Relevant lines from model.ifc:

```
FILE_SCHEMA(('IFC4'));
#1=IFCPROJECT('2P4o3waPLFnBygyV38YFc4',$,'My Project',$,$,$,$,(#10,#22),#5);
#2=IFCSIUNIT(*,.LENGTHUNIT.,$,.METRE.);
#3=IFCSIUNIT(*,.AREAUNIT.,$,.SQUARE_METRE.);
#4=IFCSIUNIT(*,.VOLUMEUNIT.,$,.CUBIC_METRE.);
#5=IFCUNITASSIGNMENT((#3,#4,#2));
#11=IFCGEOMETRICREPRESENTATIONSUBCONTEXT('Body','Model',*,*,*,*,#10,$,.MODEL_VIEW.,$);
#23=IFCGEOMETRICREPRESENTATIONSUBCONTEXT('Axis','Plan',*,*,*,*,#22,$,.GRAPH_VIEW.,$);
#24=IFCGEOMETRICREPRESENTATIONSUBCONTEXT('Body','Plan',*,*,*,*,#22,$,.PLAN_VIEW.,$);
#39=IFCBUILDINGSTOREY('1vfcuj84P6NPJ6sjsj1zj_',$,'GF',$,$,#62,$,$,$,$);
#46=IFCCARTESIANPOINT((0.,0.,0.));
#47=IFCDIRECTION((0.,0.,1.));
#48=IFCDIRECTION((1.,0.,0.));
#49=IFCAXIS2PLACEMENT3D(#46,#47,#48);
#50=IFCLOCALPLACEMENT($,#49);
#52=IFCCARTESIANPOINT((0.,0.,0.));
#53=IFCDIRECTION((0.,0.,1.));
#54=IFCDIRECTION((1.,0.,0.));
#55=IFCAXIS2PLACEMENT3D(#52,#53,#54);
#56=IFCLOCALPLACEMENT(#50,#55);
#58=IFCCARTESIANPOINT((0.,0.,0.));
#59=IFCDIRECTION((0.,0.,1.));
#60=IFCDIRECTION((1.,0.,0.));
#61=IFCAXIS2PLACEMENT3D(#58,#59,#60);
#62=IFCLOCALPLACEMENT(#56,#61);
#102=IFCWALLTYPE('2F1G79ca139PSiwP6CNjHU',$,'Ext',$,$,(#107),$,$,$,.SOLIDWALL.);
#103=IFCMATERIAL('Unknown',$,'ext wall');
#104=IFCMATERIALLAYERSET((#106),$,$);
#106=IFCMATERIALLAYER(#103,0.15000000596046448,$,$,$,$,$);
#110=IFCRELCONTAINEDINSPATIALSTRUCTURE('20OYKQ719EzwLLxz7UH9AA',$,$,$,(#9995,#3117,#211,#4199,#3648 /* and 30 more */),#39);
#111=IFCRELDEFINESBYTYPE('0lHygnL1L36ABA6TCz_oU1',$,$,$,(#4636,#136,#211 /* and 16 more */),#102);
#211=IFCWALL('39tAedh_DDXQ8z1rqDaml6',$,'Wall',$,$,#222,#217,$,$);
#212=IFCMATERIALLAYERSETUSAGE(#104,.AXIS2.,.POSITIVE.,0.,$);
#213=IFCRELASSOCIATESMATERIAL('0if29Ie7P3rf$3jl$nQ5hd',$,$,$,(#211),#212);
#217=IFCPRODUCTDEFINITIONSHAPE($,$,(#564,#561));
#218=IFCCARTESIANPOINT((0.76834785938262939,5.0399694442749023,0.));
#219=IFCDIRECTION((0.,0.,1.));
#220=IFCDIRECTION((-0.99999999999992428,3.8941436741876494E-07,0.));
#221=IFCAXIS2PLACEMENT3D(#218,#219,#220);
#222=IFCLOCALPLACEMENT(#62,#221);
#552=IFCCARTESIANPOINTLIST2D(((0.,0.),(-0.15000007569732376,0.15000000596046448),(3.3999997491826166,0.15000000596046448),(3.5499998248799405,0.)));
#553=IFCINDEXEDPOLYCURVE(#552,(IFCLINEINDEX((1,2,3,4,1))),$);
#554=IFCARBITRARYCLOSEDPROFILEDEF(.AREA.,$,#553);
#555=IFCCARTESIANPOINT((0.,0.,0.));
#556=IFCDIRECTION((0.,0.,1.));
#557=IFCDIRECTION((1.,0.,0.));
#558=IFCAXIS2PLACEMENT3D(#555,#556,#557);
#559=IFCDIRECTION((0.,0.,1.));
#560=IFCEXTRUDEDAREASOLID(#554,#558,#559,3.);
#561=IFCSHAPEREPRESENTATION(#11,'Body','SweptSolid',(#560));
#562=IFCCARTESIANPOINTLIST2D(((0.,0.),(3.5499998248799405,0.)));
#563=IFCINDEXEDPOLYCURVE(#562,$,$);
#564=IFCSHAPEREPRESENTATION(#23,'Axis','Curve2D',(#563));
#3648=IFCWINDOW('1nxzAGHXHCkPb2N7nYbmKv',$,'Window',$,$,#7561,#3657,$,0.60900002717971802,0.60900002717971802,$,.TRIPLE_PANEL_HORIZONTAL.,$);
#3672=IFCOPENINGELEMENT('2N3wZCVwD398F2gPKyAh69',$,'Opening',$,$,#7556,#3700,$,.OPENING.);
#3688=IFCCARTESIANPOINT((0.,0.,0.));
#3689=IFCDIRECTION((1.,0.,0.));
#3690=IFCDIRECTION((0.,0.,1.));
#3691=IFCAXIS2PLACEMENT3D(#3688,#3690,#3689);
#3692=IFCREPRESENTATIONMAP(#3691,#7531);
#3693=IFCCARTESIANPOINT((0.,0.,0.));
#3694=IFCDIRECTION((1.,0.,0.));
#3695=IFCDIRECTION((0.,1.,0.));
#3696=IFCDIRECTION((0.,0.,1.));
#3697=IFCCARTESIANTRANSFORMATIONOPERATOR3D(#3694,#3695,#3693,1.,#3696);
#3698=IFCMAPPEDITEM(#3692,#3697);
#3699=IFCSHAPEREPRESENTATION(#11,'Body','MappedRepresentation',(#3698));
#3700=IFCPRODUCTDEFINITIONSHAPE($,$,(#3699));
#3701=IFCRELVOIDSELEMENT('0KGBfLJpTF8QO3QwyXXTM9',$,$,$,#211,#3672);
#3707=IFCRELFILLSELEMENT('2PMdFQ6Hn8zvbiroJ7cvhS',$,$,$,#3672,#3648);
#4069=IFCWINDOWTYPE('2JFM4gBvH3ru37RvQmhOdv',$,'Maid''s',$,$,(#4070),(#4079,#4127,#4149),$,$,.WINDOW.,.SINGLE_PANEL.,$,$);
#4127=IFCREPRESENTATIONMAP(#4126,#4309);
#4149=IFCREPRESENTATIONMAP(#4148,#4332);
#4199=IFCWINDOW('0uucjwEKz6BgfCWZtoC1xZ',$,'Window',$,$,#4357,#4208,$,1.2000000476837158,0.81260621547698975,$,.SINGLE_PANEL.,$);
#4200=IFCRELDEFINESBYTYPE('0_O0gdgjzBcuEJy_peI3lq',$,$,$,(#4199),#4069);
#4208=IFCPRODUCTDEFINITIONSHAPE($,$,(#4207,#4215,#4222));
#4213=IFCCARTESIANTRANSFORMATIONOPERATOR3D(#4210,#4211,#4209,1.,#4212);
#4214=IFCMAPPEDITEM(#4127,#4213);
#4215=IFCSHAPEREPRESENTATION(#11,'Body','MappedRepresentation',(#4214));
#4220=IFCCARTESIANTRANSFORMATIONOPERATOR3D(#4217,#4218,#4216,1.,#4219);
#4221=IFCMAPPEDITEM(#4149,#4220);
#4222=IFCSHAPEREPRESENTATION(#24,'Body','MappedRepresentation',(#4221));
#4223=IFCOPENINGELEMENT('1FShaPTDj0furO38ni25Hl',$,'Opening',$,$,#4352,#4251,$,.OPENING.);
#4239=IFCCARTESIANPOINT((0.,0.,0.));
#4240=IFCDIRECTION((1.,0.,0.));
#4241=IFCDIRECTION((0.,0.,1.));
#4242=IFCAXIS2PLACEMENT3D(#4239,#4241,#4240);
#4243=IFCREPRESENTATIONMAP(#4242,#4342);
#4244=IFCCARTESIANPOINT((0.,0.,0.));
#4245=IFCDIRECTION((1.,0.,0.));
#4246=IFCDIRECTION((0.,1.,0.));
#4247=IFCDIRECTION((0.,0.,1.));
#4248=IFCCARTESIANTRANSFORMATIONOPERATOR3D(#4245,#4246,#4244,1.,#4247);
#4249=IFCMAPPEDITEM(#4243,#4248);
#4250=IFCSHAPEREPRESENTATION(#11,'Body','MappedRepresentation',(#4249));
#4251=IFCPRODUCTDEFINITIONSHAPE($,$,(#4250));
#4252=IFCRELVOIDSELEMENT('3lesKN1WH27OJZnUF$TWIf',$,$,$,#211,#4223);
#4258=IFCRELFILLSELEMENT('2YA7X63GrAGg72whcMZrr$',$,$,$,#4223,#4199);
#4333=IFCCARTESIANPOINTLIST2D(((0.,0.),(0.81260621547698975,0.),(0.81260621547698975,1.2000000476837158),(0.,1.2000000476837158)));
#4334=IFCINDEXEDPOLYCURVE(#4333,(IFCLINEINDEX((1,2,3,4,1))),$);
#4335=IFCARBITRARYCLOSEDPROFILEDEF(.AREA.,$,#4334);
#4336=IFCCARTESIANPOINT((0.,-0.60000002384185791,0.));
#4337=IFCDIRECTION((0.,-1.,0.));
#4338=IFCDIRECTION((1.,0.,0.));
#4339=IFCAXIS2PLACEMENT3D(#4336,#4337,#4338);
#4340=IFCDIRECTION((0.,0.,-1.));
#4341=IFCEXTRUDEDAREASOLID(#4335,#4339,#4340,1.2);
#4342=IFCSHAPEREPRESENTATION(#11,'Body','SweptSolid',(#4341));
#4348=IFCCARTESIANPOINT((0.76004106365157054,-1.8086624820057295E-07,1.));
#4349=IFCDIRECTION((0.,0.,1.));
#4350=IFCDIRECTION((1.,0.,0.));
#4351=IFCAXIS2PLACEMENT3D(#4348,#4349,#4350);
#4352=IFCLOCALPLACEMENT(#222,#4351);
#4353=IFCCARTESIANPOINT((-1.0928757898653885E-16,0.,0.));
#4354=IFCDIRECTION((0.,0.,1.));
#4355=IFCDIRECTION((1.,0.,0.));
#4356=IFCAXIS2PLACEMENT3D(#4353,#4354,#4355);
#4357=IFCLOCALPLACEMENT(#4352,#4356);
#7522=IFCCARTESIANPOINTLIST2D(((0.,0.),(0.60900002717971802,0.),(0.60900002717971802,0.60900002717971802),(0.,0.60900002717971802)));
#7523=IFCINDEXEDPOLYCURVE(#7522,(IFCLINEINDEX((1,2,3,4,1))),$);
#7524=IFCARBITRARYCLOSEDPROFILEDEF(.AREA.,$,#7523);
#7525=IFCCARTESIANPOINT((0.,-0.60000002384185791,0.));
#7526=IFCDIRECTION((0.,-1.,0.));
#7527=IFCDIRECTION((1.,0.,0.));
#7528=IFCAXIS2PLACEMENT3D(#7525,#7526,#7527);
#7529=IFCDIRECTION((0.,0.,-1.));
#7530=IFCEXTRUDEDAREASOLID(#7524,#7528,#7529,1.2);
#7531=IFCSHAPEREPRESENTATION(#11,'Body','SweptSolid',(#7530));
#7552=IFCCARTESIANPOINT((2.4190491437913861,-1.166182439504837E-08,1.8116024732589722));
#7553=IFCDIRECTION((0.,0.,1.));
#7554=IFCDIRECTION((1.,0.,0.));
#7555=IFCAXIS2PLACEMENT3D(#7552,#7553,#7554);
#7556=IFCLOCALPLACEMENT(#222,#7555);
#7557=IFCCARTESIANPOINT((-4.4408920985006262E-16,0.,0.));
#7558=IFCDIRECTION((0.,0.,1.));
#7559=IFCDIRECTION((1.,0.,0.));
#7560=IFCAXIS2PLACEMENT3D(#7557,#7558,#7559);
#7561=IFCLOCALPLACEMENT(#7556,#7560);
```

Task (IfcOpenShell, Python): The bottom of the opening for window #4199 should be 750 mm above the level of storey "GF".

```python
import numpy as np
import ifcopenshell
import ifcopenshell.api.geometry
import ifcopenshell.geom
import ifcopenshell.util.element
import ifcopenshell.util.placement
import ifcopenshell.util.shape
import ifcopenshell.util.unit

model = ifcopenshell.open("model.ifc")
unit_scale = ifcopenshell.util.unit.calculate_unit_scale(model)

window = model.by_id(4199)
opening = window.FillsVoids[0].RelatingOpeningElement
storey = ifcopenshell.util.element.get_container(window, ifc_class="IfcBuildingStorey")
level = ifcopenshell.util.placement.get_local_placement(storey.ObjectPlacement)[2, 3]

# The opening's origin need not be at the sill, so measure its lowest point.
shape = ifcopenshell.geom.create_shape(ifcopenshell.geom.settings(), opening)
bottom = ifcopenshell.util.shape.get_shape_bottom_elevation(shape, shape.geometry) / unit_scale
dz = level + 0.75 - bottom

shift = np.array([0.0, 0.0, dz])
# The window is placed relative to its opening, so it follows when the opening moves.
matrix = ifcopenshell.util.placement.get_local_placement(opening.ObjectPlacement)
matrix[:3, 3] += shift
ifcopenshell.api.geometry.edit_object_placement(
    model, product=opening, matrix=matrix, is_si=False, should_transform_children=True
)

print(f"moved by {dz * unit_scale:+.3f} m")

model.write("model_edited.ifc")
```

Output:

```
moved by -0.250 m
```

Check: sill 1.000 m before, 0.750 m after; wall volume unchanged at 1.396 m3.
